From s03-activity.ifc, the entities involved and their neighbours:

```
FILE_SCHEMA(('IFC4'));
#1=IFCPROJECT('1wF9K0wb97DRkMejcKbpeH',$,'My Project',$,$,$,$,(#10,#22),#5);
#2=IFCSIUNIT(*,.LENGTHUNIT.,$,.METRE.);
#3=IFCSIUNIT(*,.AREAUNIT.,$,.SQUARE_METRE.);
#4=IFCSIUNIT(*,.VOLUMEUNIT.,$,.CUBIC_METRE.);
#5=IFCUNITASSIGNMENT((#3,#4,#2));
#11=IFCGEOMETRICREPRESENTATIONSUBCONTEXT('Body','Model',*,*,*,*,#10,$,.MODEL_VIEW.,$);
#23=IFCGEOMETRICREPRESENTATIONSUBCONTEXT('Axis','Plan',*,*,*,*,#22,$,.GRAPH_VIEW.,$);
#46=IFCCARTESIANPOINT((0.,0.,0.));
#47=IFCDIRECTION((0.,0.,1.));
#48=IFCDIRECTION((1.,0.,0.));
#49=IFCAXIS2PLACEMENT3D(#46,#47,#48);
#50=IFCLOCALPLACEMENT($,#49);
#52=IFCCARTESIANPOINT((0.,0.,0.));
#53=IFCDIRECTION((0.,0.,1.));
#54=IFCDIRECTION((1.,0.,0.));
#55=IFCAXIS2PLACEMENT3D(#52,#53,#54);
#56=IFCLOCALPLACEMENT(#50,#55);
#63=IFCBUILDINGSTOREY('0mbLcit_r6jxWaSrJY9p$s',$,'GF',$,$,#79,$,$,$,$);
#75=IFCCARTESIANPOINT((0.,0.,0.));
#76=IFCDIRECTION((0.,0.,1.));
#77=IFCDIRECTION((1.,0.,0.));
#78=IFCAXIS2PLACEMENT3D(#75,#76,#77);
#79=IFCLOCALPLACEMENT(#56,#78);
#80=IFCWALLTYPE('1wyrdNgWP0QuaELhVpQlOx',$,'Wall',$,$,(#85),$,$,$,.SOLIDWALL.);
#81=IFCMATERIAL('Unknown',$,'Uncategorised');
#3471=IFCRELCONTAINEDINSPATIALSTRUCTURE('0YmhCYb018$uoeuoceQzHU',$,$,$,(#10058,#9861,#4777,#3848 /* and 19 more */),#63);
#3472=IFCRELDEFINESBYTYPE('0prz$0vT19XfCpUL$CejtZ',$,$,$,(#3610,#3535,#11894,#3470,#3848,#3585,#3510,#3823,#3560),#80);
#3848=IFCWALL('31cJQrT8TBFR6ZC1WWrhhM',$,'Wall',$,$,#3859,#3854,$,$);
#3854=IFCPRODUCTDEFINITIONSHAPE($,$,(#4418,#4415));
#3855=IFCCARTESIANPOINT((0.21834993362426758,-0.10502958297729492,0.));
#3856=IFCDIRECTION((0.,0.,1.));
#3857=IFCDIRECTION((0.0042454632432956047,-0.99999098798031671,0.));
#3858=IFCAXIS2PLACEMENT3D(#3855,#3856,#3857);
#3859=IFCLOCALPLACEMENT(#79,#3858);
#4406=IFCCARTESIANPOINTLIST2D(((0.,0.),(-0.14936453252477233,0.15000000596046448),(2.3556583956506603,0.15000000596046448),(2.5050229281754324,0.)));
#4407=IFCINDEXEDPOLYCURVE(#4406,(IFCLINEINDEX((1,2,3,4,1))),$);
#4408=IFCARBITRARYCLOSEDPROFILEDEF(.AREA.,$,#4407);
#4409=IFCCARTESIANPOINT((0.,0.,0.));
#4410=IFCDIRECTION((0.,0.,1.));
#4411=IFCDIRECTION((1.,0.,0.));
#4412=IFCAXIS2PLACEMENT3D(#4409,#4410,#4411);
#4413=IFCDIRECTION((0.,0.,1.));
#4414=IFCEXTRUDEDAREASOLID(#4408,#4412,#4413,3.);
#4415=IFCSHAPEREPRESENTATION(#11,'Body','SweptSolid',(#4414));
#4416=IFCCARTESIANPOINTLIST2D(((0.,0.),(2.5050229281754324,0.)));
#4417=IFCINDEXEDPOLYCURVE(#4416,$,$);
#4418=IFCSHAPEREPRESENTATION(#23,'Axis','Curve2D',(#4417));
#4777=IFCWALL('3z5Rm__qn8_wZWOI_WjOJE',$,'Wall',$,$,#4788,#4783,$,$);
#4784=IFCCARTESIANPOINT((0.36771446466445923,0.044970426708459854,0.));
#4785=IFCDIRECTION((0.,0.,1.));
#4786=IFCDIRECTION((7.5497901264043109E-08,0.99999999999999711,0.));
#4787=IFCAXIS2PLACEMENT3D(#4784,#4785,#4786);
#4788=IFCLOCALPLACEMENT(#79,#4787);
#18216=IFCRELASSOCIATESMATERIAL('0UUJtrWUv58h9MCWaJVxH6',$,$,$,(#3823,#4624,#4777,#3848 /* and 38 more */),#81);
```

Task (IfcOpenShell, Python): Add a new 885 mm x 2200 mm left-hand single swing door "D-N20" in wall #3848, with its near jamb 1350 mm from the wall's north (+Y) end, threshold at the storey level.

```python
import numpy as np
import ifcopenshell
import ifcopenshell.api.feature
import ifcopenshell.api.geometry
import ifcopenshell.api.root
import ifcopenshell.api.spatial
import ifcopenshell.geom
import ifcopenshell.util.element
import ifcopenshell.util.placement
import ifcopenshell.util.representation
import ifcopenshell.util.shape
import ifcopenshell.util.unit

model = ifcopenshell.open("s03-activity.ifc")
unit_scale = ifcopenshell.util.unit.calculate_unit_scale(model)
settings = ifcopenshell.geom.settings()


def volume(element):
    """Net volume in cubic metres, openings subtracted."""
    shape = ifcopenshell.geom.create_shape(settings, element)
    return ifcopenshell.util.shape.get_volume(shape.geometry)


wall = model.by_guid("31cJQrT8TBFR6ZC1WWrhhM")
storey = ifcopenshell.util.element.get_container(wall, ifc_class="IfcBuildingStorey")
context = ifcopenshell.util.representation.get_context(model, "Model", "Body", "MODEL_VIEW")
before = volume(wall)

width, height, from_end, sill = 0.885, 2.2, 1.35, 0.0  # metres

# The wall runs along its own X axis, and the end named is its -X end.
wall_shape = ifcopenshell.geom.create_shape(settings, wall)
x, y, z = ifcopenshell.util.shape.get_vertices(wall_shape.geometry).T
start = x.min() + from_end
face, thickness = float(y.min()), float(y.max() - y.min())
wall_matrix = ifcopenshell.util.placement.get_local_placement(wall.ObjectPlacement)
level = ifcopenshell.util.placement.get_local_placement(storey.ObjectPlacement)[2, 3]


def in_wall(x, y):
    """Placement at x, y metres in the wall's axes, at sill height."""
    matrix = wall_matrix.copy()
    matrix[:, 3] = wall_matrix @ np.array([x / unit_scale, y / unit_scale, 0.0, 1.0])
    matrix[2, 3] = level + sill / unit_scale
    return matrix


# Opening: a box that overshoots both wall faces by 50 mm.
opening = ifcopenshell.api.root.create_entity(model, ifc_class="IfcOpeningElement", predefined_type="OPENING")
box = ifcopenshell.api.geometry.add_wall_representation(
    model, context=context, length=width, height=height, thickness=thickness + 0.1
)
ifcopenshell.api.geometry.assign_representation(model, product=opening, representation=box)
ifcopenshell.api.geometry.edit_object_placement(model, product=opening, matrix=in_wall(start, face - 0.05), is_si=False)
ifcopenshell.api.feature.add_feature(model, feature=opening, element=wall)

door = ifcopenshell.api.root.create_entity(model, ifc_class="IfcDoor", name="D-N20", predefined_type="DOOR")
door.OverallWidth, door.OverallHeight = width / unit_scale, height / unit_scale
door.OperationType = "SINGLE_SWING_LEFT"
body = ifcopenshell.api.geometry.add_door_representation(
    model,
    context=context,
    overall_width=door.OverallWidth,
    overall_height=door.OverallHeight,
    operation_type="SINGLE_SWING_LEFT",
    lining_properties={"LiningDepth": thickness / unit_scale, "ThresholdDepth": thickness / unit_scale},
)
ifcopenshell.api.geometry.assign_representation(model, product=door, representation=body)
ifcopenshell.api.spatial.assign_container(model, products=[door], relating_structure=storey)
ifcopenshell.api.feature.add_filling(model, opening=opening, element=door)

# The lining spans the wall, so the door starts at the wall face.
ifcopenshell.api.geometry.edit_object_placement(model, product=door, matrix=in_wall(start, face), is_si=False)

after = volume(wall)

print(f"wall volume {before:.3f} -> {after:.3f} m3")

model.write("s03-activity_updated.ifc")
```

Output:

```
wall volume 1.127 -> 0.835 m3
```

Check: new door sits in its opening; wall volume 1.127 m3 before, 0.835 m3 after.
